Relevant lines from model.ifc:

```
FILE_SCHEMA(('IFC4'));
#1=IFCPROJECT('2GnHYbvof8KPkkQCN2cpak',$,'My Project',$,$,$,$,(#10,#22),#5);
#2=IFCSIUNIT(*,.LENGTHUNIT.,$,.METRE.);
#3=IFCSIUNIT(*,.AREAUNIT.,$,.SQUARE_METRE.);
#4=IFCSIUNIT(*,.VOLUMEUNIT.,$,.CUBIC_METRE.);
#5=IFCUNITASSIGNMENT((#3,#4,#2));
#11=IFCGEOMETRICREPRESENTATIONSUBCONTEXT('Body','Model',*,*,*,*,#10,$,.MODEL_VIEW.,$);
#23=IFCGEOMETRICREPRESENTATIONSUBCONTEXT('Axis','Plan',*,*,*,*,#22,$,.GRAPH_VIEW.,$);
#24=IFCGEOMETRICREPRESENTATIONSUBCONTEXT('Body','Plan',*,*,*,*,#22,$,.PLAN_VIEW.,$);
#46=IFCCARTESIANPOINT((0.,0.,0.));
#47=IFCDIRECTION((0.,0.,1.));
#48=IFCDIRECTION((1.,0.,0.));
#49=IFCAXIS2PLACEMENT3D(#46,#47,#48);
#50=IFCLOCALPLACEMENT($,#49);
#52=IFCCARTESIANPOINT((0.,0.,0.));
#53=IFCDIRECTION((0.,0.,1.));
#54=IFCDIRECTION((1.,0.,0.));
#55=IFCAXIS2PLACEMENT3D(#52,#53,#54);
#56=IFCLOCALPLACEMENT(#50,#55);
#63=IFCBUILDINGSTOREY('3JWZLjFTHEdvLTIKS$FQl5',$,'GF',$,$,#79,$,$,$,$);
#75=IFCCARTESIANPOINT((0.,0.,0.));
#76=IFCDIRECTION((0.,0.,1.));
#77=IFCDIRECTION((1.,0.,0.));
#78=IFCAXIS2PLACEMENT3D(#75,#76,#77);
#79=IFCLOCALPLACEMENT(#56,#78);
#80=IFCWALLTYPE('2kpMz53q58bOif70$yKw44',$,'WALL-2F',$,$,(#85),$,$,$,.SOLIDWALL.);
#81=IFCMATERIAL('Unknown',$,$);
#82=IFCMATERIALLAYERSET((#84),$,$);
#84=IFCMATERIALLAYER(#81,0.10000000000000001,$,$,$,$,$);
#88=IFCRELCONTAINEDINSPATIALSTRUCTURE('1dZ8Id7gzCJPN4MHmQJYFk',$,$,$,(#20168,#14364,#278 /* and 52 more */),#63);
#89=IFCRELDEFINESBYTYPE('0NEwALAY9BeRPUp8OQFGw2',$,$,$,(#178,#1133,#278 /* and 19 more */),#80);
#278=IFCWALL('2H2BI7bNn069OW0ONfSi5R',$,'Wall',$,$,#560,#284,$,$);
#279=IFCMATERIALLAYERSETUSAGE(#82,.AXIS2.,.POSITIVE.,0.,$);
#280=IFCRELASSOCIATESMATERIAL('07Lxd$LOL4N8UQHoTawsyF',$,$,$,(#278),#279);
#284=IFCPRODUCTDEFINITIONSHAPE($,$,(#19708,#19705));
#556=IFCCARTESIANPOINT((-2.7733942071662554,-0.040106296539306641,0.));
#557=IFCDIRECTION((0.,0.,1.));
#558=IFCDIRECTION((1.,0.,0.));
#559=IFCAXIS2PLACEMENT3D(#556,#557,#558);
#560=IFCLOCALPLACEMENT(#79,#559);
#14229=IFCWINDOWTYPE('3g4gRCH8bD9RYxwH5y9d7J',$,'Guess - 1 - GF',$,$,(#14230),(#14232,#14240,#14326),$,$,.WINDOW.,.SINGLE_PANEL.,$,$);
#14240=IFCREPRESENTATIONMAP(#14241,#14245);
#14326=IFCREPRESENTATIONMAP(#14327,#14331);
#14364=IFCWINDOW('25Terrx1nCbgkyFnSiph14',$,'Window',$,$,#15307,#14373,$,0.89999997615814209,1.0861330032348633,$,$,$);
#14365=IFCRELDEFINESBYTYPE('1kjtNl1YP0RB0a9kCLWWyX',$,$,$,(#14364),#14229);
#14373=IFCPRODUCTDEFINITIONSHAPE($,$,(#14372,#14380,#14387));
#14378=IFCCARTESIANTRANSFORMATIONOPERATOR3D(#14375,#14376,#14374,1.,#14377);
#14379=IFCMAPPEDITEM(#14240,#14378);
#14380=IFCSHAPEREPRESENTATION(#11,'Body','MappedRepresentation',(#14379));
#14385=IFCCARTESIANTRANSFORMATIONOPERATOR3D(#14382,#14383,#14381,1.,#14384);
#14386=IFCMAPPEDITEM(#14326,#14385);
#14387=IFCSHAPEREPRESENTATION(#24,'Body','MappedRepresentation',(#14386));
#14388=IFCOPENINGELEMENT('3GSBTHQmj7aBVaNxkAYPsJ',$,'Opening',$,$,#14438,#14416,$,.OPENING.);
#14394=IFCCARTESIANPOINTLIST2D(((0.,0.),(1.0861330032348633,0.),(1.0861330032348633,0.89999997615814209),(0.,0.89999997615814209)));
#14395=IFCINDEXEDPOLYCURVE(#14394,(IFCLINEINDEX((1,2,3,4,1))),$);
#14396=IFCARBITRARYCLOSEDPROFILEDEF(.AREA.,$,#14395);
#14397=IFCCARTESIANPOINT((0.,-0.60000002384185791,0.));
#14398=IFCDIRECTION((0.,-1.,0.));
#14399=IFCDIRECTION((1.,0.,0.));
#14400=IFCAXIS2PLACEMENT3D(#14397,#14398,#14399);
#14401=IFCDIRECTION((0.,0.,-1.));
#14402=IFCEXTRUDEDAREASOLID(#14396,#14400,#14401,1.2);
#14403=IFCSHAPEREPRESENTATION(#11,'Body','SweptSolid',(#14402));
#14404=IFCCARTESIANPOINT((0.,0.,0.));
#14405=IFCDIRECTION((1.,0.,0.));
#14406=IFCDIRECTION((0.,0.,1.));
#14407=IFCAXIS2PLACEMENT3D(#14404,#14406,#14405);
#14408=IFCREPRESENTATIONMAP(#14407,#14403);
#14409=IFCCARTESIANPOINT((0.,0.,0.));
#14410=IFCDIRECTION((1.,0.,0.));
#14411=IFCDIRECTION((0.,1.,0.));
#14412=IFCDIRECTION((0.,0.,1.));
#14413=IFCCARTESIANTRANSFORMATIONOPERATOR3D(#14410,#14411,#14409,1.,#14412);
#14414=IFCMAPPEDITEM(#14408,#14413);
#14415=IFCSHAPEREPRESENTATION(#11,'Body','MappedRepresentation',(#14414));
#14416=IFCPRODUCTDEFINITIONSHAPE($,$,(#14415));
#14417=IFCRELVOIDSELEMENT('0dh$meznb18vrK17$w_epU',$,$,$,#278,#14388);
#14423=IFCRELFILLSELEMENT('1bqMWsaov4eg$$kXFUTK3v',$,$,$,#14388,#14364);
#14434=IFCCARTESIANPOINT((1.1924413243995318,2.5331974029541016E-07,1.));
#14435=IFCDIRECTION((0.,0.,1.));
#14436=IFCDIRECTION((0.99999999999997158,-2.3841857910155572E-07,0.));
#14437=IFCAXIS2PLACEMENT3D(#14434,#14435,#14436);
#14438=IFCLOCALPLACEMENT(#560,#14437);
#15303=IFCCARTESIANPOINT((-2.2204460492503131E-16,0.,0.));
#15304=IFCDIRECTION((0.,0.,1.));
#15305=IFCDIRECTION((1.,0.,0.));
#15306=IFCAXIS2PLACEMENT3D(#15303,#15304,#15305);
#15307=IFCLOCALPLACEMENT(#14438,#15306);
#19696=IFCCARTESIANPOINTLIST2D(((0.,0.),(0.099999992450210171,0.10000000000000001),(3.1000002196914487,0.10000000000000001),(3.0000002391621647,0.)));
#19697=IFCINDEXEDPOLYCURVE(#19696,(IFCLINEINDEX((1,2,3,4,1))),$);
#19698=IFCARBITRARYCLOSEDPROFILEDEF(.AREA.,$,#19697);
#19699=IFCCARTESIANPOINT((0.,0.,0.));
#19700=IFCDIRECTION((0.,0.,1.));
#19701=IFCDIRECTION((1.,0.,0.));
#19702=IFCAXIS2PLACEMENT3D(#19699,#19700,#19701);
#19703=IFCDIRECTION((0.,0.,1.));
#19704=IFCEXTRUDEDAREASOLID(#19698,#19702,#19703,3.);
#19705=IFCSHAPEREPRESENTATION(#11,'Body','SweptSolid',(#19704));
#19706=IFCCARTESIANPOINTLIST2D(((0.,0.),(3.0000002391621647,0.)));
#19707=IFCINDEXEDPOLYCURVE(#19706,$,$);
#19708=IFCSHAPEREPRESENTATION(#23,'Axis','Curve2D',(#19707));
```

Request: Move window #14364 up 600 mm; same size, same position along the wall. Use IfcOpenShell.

```python
import numpy as np
import ifcopenshell
import ifcopenshell.api.geometry
import ifcopenshell.util.placement
import ifcopenshell.util.unit

model = ifcopenshell.open("model.ifc")
unit_scale = ifcopenshell.util.unit.calculate_unit_scale(model)

window = model.by_guid("25Terrx1nCbgkyFnSiph14")
opening = window.FillsVoids[0].RelatingOpeningElement
dz = 0.6

shift = np.array([0.0, 0.0, dz])
# The window is placed relative to its opening, so it follows when the opening moves.
matrix = ifcopenshell.util.placement.get_local_placement(opening.ObjectPlacement)
matrix[:3, 3] += shift
ifcopenshell.api.geometry.edit_object_placement(
    model, product=opening, matrix=matrix, is_si=False, should_transform_children=True
)

print(f"moved by {dz * unit_scale:+.3f} m")

model.write("model_rev.ifc")
```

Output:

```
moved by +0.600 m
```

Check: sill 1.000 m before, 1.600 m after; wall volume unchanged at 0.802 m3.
